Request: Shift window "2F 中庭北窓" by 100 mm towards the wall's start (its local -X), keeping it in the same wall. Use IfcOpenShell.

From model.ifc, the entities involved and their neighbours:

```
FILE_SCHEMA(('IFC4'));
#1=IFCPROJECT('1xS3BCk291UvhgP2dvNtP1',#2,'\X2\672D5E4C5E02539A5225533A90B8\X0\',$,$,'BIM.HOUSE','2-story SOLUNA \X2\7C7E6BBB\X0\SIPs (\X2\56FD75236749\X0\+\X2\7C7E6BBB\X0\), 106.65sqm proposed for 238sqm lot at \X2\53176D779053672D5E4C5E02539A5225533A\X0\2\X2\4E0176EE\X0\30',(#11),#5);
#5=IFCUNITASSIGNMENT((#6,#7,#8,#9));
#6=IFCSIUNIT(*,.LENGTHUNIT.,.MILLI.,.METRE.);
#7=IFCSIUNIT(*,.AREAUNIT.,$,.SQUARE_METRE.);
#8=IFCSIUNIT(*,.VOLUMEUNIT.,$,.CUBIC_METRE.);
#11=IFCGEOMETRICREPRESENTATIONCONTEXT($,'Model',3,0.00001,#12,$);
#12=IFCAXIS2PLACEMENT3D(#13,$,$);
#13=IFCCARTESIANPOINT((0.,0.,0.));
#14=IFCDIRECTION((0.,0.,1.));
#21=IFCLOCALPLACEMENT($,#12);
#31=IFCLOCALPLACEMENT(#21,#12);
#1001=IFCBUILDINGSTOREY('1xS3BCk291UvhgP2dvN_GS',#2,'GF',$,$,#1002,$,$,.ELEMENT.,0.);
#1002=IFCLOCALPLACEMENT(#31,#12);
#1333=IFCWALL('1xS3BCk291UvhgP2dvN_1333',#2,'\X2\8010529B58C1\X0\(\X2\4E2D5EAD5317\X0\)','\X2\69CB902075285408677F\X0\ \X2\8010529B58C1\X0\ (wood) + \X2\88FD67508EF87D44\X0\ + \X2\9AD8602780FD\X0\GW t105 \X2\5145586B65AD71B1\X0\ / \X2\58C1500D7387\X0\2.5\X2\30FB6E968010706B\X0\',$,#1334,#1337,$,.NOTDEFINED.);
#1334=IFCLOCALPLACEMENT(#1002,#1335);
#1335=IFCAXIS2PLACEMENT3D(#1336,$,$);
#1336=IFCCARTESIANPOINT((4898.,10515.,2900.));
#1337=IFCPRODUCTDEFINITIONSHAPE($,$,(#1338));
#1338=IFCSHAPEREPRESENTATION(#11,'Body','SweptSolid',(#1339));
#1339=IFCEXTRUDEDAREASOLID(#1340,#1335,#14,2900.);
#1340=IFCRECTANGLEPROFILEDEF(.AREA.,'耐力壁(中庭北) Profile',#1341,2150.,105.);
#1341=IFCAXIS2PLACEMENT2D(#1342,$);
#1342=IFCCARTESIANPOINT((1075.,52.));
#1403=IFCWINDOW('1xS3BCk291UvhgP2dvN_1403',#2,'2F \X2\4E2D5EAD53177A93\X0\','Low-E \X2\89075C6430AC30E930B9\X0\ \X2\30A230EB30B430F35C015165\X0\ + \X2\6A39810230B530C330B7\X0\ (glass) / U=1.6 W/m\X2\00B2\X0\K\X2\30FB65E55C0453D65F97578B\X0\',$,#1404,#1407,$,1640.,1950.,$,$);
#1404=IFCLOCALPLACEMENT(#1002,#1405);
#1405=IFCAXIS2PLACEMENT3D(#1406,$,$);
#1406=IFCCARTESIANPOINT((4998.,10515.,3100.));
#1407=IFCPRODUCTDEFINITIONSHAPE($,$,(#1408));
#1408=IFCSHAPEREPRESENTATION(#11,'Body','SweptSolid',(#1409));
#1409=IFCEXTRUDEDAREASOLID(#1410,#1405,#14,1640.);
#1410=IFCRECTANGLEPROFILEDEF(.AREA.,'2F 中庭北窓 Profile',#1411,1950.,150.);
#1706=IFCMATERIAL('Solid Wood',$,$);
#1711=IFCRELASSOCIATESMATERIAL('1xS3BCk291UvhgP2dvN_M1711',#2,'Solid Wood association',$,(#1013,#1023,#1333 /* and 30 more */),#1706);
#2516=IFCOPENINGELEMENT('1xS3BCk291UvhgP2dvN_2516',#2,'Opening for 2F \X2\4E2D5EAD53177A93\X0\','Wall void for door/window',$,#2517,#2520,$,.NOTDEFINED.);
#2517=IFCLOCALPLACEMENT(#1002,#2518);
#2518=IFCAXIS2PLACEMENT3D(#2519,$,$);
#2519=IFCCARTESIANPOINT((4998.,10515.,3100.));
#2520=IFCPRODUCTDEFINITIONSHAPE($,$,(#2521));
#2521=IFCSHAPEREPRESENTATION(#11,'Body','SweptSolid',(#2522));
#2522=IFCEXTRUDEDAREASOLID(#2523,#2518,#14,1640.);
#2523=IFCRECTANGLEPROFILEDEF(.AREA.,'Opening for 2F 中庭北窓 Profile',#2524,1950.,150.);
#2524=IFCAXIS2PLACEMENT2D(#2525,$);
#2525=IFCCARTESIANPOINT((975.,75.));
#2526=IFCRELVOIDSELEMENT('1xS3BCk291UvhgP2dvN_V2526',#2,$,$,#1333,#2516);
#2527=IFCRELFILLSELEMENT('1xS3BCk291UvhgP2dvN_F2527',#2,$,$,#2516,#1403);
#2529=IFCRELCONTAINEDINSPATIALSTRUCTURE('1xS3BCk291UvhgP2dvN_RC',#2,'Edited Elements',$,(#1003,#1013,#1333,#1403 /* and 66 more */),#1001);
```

```python
import ifcopenshell
import ifcopenshell.api.geometry
import ifcopenshell.util.placement
import ifcopenshell.util.unit

model = ifcopenshell.open("model.ifc")
unit_scale = ifcopenshell.util.unit.calculate_unit_scale(model)

window = model.by_id(1403)
opening = window.FillsVoids[0].RelatingOpeningElement
wall = opening.VoidsElements[0].RelatingBuildingElement

wall_matrix = ifcopenshell.util.placement.get_local_placement(wall.ObjectPlacement)
shift = wall_matrix[:3, 0] * -0.1 / unit_scale
before = ifcopenshell.util.placement.get_local_placement(window.ObjectPlacement)[:3, 3].copy()

# The window is not placed relative to its opening, so move both.
for product in (opening, window):
    matrix = ifcopenshell.util.placement.get_local_placement(product.ObjectPlacement)
    matrix[:3, 3] += shift
    ifcopenshell.api.geometry.edit_object_placement(model, product=product, matrix=matrix, is_si=False)

after = ifcopenshell.util.placement.get_local_placement(window.ObjectPlacement)[:3, 3]
print("window moved by", (after - before).round(3) + 0.0)

model.write("model_updated.ifc")
```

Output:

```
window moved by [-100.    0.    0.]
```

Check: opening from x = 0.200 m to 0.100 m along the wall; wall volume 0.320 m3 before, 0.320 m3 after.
